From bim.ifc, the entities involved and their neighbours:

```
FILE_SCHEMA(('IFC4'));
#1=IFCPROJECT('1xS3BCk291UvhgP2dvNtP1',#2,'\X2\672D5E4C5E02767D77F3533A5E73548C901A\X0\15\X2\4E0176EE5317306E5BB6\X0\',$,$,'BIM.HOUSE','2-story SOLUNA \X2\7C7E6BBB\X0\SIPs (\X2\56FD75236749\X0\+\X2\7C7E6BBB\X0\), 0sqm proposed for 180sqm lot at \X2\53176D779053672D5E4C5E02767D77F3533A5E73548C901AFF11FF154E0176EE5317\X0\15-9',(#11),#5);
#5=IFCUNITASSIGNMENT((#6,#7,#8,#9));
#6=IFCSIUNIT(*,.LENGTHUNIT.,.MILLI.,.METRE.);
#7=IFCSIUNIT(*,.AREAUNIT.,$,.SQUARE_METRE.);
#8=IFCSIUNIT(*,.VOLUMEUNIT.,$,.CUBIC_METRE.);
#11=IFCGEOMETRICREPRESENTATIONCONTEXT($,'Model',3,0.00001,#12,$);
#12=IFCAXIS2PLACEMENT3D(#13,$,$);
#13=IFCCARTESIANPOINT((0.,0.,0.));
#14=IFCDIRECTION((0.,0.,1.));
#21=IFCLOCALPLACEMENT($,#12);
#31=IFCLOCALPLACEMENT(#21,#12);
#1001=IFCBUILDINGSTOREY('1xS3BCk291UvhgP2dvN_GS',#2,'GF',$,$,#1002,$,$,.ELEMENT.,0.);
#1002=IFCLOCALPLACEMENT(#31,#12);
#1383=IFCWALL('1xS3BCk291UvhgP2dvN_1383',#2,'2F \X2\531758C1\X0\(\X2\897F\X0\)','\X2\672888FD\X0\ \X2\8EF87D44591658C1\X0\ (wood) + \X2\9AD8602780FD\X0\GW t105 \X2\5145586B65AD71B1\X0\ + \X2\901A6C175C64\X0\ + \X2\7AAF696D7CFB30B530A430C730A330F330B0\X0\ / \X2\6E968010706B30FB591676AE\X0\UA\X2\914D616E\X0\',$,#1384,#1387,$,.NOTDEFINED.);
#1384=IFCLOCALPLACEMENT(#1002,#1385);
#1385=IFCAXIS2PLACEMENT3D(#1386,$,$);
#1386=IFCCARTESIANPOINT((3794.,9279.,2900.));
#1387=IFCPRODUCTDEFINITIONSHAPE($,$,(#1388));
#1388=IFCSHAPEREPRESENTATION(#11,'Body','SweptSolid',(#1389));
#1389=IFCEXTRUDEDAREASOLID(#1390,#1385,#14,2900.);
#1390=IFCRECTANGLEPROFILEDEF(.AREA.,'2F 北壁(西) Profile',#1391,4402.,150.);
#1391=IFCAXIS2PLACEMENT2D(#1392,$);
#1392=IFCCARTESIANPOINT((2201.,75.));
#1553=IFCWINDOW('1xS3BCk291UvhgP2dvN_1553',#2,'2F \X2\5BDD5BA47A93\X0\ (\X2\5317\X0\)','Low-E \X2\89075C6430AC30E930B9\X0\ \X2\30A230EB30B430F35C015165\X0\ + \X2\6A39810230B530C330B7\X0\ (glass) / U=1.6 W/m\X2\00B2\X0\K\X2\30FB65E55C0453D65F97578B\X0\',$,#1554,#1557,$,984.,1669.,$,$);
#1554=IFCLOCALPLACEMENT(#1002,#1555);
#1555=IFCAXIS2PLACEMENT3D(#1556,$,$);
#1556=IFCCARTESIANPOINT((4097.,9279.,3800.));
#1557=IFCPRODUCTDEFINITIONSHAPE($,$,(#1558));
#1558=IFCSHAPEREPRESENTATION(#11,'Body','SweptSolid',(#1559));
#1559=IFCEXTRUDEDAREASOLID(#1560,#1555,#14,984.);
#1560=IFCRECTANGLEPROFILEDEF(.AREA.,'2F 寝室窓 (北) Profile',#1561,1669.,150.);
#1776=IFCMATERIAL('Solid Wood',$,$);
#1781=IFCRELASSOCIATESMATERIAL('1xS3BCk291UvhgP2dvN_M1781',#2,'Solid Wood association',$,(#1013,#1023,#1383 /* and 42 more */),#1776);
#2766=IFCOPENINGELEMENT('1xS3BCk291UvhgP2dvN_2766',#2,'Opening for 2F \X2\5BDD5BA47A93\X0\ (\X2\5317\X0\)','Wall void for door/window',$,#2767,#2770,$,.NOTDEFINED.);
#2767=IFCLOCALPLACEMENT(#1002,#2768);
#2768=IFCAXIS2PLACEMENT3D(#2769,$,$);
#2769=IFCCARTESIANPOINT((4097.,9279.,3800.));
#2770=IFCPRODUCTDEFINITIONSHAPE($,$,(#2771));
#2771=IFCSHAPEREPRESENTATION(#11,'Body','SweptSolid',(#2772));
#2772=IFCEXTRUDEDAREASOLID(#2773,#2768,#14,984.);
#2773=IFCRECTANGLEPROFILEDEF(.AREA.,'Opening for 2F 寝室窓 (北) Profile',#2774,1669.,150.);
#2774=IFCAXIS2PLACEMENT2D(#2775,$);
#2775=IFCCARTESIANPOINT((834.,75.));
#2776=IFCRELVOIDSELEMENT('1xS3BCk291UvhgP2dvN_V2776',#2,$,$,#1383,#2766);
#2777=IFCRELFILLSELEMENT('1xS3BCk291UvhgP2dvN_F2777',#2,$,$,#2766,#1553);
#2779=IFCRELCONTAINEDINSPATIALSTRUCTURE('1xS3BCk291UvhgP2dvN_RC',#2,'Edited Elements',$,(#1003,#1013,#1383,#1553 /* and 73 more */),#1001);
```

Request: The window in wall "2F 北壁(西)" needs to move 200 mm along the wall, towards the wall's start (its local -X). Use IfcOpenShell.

```python
import ifcopenshell
import ifcopenshell.api.geometry
import ifcopenshell.util.placement

model = ifcopenshell.open("bim.ifc")

window = model.by_guid("1xS3BCk291UvhgP2dvN_1553")
opening = window.FillsVoids[0].RelatingOpeningElement
wall = opening.VoidsElements[0].RelatingBuildingElement

wall_matrix = ifcopenshell.util.placement.get_local_placement(wall.ObjectPlacement)
shift = wall_matrix[:3, 0] * -200.0
before = ifcopenshell.util.placement.get_local_placement(window.ObjectPlacement)[:3, 3].copy()

# The window is not placed relative to its opening, so move both.
for product in (opening, window):
    matrix = ifcopenshell.util.placement.get_local_placement(product.ObjectPlacement)
    matrix[:3, 3] += shift
    ifcopenshell.api.geometry.edit_object_placement(model, product=product, matrix=matrix, is_si=False)

after = ifcopenshell.util.placement.get_local_placement(window.ObjectPlacement)[:3, 3]
print("window moved by", (after - before).round(3) + 0.0)

model.write("bim_edited.ifc")
```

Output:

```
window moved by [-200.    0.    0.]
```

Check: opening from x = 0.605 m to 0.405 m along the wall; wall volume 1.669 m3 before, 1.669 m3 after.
